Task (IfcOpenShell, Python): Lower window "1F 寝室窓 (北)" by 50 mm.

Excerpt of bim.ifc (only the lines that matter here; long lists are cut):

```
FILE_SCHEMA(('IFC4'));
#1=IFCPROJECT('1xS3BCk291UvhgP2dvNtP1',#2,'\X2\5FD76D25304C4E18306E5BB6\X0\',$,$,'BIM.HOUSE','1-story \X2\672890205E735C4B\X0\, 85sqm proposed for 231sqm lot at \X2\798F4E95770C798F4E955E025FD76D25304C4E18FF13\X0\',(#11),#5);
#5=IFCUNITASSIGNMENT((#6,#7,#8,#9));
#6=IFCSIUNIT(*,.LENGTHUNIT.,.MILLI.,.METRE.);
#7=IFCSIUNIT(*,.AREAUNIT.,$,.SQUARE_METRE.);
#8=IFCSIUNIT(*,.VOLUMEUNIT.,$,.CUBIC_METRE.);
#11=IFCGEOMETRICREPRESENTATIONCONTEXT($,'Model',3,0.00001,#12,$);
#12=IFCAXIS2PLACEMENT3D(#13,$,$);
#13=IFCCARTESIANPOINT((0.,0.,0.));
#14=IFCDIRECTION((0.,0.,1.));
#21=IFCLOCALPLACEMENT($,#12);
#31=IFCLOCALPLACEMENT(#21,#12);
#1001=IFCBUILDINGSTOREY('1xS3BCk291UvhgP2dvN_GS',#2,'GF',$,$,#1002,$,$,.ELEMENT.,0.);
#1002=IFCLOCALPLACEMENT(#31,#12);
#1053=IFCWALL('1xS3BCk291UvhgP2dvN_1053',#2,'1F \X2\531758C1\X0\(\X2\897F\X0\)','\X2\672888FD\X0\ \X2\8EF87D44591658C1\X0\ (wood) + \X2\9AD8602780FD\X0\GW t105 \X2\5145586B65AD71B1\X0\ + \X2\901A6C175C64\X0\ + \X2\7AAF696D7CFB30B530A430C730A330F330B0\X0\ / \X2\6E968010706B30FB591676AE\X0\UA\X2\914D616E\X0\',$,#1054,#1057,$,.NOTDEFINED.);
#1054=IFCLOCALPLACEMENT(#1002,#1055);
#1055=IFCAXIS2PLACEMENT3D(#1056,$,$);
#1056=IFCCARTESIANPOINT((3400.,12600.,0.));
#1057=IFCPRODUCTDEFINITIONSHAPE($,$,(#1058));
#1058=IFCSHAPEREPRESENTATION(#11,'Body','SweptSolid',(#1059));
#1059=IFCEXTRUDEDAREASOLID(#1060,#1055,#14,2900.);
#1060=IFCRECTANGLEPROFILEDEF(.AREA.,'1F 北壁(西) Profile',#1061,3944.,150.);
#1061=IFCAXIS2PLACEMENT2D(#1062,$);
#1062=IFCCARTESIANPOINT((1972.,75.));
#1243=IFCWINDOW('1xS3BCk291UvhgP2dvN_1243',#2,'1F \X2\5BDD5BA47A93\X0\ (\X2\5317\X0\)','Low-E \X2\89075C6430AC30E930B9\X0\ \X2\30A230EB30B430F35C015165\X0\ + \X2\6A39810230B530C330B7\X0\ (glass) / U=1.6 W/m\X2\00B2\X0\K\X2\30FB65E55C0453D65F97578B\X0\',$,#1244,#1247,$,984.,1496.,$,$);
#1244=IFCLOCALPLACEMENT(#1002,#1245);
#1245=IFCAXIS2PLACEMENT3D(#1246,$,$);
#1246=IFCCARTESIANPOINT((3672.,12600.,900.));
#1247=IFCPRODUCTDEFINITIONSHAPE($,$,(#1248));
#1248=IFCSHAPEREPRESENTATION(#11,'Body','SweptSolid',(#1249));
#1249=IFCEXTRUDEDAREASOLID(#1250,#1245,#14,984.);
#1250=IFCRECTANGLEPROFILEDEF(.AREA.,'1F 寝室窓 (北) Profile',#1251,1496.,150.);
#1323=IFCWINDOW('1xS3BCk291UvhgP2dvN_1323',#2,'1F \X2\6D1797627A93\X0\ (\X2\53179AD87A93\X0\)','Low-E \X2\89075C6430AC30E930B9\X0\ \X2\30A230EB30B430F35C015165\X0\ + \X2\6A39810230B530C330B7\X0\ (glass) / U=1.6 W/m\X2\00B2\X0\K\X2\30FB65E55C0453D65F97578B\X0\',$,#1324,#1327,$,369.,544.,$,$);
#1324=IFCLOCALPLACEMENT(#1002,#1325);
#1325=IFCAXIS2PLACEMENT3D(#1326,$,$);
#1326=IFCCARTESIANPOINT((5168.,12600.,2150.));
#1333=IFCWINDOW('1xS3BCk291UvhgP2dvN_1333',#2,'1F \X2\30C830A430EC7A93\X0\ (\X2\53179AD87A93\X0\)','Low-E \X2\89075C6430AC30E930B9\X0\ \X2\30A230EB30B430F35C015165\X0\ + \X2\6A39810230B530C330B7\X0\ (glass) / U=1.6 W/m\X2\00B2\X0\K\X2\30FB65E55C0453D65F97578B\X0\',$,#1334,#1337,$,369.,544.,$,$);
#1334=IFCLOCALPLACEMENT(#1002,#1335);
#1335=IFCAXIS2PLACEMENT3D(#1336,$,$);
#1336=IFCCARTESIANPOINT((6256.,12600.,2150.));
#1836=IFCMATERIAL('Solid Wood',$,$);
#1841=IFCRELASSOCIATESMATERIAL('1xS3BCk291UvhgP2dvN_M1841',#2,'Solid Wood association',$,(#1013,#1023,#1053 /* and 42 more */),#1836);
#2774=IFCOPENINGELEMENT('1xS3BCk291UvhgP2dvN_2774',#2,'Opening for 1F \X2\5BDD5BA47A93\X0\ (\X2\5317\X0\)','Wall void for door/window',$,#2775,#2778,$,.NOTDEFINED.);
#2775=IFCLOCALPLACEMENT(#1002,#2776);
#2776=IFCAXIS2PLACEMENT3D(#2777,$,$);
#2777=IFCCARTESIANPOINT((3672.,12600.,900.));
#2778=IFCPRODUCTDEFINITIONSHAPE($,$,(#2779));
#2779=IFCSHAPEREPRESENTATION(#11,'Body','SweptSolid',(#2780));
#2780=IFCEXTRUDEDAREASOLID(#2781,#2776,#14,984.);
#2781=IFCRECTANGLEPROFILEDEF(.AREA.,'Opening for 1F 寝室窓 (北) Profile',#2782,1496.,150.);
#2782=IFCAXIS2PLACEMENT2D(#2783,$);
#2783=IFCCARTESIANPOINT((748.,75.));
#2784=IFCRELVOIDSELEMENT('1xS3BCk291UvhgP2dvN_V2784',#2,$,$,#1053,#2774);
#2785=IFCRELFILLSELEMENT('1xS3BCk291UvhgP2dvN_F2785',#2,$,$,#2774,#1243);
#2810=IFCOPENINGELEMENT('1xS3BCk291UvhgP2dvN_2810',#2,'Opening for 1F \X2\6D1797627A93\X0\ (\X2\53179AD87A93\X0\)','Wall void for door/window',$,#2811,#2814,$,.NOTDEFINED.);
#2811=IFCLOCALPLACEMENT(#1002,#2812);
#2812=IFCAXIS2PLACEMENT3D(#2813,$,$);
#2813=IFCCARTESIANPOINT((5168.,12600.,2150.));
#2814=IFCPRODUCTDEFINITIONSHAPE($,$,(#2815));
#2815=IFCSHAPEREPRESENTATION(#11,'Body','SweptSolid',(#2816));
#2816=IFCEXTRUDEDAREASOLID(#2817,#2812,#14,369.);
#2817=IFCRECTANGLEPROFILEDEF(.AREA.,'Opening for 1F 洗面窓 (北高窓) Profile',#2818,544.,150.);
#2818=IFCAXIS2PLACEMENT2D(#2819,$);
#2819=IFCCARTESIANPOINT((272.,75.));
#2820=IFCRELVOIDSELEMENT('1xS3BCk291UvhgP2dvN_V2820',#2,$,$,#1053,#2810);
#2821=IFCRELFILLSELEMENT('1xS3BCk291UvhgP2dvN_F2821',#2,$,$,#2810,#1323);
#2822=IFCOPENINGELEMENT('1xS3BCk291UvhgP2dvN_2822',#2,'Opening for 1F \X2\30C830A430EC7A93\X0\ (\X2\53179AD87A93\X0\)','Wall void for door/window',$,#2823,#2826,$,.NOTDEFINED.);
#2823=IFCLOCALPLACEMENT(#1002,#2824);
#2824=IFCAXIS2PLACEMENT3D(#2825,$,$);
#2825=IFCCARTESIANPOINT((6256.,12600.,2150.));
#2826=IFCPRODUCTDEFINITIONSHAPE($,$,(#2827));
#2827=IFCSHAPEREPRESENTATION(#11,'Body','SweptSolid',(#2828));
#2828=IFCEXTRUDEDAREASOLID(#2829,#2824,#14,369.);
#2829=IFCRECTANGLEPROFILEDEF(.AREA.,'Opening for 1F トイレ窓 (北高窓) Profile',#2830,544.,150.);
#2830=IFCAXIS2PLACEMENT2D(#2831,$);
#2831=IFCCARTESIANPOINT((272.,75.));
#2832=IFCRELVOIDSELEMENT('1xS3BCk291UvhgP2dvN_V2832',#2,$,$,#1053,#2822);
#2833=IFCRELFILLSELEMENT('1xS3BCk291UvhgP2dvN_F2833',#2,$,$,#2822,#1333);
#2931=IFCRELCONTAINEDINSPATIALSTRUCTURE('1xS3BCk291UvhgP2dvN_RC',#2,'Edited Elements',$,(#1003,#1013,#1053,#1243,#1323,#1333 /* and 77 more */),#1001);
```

```python
import numpy as np
import ifcopenshell
import ifcopenshell.api.geometry
import ifcopenshell.util.placement
import ifcopenshell.util.unit

model = ifcopenshell.open("bim.ifc")
unit_scale = ifcopenshell.util.unit.calculate_unit_scale(model)

window = model.by_guid("1xS3BCk291UvhgP2dvN_1243")
opening = window.FillsVoids[0].RelatingOpeningElement
dz = -0.05 / unit_scale

shift = np.array([0.0, 0.0, dz])
# The window is not placed relative to its opening, so move both.
for product in (opening, window):
    matrix = ifcopenshell.util.placement.get_local_placement(product.ObjectPlacement)
    matrix[:3, 3] += shift
    ifcopenshell.api.geometry.edit_object_placement(model, product=product, matrix=matrix, is_si=False)

print(f"moved by {dz * unit_scale:+.3f} m")

model.write("bim_v2.ifc")
```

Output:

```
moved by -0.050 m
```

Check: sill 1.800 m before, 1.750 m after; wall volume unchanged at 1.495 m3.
